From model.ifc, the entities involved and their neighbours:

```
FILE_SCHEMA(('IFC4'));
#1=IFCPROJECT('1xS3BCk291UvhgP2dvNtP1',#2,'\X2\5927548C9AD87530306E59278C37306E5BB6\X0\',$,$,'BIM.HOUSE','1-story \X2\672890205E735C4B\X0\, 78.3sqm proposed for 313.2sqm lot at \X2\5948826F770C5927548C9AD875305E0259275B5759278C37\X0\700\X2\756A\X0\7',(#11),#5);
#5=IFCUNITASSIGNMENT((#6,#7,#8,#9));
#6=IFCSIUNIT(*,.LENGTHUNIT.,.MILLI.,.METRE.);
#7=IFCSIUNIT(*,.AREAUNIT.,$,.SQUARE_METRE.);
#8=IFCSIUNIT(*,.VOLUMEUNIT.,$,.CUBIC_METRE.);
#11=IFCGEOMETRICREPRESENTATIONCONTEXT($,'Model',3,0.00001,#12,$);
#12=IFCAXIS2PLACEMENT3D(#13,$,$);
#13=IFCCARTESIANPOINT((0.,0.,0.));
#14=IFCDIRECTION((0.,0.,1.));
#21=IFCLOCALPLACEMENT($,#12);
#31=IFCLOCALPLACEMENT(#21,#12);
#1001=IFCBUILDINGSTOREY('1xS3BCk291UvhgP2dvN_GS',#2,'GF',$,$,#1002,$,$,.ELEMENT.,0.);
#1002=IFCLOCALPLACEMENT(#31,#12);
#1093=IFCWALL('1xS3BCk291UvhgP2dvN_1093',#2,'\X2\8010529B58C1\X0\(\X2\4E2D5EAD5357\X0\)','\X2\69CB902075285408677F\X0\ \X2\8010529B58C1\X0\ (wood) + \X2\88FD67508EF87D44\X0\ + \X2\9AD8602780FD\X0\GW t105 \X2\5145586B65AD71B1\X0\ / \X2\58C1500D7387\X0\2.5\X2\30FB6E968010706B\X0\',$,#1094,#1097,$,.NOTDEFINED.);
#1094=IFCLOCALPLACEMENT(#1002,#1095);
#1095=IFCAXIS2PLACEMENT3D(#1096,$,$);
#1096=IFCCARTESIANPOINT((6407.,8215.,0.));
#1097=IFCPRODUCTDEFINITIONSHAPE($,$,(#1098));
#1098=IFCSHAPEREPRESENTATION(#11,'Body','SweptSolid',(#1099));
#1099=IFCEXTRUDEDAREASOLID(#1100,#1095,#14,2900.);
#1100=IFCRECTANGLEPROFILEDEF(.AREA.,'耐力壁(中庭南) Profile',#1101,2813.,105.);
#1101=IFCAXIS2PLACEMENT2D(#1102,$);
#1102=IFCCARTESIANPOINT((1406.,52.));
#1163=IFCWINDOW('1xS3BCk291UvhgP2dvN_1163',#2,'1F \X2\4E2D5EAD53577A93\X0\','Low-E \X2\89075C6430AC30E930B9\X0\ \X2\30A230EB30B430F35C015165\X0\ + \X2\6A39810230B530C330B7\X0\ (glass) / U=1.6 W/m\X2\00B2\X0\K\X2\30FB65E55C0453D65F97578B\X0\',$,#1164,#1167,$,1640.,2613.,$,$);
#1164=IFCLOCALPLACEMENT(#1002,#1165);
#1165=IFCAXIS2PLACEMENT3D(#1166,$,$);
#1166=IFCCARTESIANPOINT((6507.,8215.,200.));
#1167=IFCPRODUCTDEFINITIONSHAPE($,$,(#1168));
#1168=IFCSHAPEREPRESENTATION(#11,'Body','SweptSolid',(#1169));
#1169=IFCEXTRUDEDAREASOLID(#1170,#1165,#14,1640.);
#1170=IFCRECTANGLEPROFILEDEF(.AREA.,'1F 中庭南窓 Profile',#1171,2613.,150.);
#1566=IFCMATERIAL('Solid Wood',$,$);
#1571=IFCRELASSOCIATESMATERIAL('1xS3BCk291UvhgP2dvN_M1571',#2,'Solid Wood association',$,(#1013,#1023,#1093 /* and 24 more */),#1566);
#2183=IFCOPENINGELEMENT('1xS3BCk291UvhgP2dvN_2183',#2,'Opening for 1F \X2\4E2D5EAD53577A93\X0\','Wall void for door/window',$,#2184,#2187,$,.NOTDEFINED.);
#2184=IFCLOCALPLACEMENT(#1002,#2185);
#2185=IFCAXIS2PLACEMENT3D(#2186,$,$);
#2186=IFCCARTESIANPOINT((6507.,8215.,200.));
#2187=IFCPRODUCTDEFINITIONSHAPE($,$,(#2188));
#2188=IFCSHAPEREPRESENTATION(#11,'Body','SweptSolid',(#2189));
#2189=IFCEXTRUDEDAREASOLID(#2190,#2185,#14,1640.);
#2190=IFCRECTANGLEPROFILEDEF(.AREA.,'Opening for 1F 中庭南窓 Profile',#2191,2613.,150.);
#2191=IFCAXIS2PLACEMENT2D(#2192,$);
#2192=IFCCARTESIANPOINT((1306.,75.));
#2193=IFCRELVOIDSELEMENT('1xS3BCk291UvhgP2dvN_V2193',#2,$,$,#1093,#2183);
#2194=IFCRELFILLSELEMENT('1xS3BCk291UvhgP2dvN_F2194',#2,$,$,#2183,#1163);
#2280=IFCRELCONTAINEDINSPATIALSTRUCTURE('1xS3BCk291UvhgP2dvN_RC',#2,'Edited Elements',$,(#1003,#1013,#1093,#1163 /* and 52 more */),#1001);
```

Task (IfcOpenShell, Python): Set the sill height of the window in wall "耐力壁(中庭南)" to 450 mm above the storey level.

```python
import numpy as np
import ifcopenshell
import ifcopenshell.api.geometry
import ifcopenshell.geom
import ifcopenshell.util.element
import ifcopenshell.util.placement
import ifcopenshell.util.shape
import ifcopenshell.util.unit

model = ifcopenshell.open("model.ifc")
unit_scale = ifcopenshell.util.unit.calculate_unit_scale(model)

window = model.by_id(1163)
opening = window.FillsVoids[0].RelatingOpeningElement
storey = ifcopenshell.util.element.get_container(window, ifc_class="IfcBuildingStorey")
level = ifcopenshell.util.placement.get_local_placement(storey.ObjectPlacement)[2, 3]

# The opening's origin need not be at the sill, so measure its lowest point.
shape = ifcopenshell.geom.create_shape(ifcopenshell.geom.settings(), opening)
bottom = ifcopenshell.util.shape.get_shape_bottom_elevation(shape, shape.geometry) / unit_scale
dz = level + 0.45 / unit_scale - bottom

shift = np.array([0.0, 0.0, dz])
# The window is not placed relative to its opening, so move both.
for product in (opening, window):
    matrix = ifcopenshell.util.placement.get_local_placement(product.ObjectPlacement)
    matrix[:3, 3] += shift
    ifcopenshell.api.geometry.edit_object_placement(model, product=product, matrix=matrix, is_si=False)

print(f"moved by {dz * unit_scale:+.3f} m")

model.write("model_updated.ifc")
```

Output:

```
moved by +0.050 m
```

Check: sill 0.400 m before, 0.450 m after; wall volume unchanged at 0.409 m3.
